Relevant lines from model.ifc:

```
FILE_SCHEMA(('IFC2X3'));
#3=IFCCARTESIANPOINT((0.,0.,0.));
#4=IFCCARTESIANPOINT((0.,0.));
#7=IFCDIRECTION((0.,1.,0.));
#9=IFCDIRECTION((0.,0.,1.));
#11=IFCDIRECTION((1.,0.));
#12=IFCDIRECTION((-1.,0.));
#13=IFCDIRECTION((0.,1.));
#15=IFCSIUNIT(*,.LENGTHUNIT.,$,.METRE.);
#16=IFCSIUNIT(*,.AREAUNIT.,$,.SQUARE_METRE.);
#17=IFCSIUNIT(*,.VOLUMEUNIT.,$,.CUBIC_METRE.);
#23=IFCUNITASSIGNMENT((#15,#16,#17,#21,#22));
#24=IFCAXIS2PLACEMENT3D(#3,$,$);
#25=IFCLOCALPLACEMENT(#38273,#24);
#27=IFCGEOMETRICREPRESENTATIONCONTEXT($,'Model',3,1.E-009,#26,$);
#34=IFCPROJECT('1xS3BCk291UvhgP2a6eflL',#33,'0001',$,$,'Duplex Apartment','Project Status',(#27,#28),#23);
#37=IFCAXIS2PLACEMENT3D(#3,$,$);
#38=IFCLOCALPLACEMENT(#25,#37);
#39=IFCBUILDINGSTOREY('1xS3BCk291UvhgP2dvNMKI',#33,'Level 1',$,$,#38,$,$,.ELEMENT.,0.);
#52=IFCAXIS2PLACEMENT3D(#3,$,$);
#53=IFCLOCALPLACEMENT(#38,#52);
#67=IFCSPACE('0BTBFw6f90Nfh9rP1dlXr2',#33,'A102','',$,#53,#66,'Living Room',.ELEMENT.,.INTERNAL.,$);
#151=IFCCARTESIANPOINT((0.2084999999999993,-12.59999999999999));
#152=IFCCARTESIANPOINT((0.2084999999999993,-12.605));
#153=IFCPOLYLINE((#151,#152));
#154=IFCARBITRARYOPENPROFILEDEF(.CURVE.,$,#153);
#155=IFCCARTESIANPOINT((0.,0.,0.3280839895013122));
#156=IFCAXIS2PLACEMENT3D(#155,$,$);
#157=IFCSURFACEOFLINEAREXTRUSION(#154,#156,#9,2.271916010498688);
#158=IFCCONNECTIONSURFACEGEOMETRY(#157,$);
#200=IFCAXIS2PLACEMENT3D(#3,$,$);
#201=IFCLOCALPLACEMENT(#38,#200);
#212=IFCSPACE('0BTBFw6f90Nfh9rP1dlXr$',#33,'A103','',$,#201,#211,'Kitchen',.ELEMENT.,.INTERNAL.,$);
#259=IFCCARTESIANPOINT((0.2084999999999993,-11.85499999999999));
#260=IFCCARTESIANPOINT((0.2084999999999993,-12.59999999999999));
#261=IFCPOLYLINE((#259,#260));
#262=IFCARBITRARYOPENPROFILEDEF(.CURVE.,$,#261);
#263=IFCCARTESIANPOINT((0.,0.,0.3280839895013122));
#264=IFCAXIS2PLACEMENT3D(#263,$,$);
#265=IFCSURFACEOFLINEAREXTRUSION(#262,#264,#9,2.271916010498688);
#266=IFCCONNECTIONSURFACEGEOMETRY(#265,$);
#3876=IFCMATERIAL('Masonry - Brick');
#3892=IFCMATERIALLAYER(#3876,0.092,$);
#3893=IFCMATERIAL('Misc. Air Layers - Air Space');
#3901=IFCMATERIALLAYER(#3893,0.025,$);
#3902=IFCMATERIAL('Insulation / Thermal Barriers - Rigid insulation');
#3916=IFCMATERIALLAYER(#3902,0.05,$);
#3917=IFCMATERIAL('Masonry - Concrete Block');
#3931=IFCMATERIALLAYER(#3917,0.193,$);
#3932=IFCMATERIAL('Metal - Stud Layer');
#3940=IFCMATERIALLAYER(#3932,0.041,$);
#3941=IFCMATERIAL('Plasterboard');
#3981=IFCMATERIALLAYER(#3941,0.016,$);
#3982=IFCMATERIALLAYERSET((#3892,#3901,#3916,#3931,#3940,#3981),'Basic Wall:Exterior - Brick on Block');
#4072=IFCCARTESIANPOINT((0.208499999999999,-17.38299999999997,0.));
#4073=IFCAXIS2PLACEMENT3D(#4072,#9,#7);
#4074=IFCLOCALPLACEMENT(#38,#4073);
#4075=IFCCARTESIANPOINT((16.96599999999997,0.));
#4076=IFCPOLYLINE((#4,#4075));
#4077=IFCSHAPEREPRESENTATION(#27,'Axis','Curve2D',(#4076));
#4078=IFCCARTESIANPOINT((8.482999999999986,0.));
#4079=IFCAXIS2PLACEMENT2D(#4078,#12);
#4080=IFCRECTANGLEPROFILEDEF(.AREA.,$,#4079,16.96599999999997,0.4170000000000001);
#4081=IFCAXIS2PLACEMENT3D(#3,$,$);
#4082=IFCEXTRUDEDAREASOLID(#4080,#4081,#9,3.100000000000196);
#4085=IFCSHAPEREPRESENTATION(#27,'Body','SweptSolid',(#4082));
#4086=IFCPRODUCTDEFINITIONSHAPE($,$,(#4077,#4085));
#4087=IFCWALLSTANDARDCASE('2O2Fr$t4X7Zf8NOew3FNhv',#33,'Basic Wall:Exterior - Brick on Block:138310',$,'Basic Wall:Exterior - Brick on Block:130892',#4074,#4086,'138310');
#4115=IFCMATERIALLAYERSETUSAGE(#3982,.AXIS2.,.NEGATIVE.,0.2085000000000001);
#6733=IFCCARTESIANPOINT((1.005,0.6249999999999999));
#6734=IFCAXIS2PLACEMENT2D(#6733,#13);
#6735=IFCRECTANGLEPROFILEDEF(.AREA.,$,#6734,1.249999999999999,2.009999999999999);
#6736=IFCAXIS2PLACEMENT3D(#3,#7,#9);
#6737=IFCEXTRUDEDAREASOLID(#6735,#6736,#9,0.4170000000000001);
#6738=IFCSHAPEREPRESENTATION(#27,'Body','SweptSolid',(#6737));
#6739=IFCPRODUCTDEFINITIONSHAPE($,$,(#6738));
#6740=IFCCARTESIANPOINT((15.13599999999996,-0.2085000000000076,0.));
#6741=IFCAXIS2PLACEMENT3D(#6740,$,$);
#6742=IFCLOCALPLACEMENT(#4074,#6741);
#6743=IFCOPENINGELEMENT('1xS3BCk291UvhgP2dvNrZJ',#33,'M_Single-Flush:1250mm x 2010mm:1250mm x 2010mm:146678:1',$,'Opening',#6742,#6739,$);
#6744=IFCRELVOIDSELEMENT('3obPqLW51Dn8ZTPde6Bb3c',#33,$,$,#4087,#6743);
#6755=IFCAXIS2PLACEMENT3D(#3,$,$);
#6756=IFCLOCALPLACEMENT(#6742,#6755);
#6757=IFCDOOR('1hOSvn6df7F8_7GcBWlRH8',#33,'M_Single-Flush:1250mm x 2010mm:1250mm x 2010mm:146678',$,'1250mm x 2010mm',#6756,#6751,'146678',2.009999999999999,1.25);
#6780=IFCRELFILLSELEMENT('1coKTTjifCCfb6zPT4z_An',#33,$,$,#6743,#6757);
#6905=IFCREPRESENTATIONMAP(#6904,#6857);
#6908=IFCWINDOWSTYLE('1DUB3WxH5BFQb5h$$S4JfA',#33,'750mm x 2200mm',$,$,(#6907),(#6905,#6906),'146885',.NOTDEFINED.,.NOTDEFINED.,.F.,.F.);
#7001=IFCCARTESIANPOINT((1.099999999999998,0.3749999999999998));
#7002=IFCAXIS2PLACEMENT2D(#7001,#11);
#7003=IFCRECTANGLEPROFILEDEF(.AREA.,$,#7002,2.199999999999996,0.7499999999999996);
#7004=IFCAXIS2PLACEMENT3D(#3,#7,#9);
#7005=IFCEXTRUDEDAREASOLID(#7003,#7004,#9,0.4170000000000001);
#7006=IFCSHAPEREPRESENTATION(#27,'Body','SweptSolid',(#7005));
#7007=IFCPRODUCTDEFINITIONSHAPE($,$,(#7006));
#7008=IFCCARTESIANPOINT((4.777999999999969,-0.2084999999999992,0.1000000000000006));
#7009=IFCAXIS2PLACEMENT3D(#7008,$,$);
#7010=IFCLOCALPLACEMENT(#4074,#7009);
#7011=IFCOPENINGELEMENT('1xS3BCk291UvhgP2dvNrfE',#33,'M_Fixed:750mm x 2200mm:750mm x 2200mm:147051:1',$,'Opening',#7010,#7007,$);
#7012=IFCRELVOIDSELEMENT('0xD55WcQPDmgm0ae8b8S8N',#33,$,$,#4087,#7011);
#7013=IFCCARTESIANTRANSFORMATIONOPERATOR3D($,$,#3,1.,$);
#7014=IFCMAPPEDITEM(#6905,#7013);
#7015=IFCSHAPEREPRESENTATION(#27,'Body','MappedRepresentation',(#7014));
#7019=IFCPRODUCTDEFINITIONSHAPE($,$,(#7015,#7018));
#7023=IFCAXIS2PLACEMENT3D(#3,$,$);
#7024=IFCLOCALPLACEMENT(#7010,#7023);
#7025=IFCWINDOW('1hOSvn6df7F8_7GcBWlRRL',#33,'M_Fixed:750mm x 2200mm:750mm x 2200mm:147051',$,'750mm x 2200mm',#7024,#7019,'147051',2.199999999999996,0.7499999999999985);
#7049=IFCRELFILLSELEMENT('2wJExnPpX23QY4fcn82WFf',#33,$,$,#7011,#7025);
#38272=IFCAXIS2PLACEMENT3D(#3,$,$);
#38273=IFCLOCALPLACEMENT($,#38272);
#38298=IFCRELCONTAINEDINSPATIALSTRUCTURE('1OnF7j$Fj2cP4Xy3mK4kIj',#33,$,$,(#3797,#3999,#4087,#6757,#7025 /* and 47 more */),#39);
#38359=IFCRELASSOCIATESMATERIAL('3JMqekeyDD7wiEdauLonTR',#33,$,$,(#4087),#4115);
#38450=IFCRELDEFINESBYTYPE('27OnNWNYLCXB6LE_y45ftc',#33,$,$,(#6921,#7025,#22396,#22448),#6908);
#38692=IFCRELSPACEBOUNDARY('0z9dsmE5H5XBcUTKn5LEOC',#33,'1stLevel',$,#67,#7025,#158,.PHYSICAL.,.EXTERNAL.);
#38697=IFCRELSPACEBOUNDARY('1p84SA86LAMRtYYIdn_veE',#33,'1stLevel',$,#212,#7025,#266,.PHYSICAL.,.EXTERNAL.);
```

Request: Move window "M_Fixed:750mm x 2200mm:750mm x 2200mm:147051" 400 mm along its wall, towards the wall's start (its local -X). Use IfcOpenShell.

```python
import numpy as np
import ifcopenshell
import ifcopenshell.api.geometry
import ifcopenshell.util.placement
import ifcopenshell.util.unit

model = ifcopenshell.open("model.ifc")
unit_scale = ifcopenshell.util.unit.calculate_unit_scale(model)

window = model.by_id(7025)
opening = window.FillsVoids[0].RelatingOpeningElement
wall = opening.VoidsElements[0].RelatingBuildingElement

wall_matrix = ifcopenshell.util.placement.get_local_placement(wall.ObjectPlacement)
shift = wall_matrix[:3, 0] * -0.4 / unit_scale
before = ifcopenshell.util.placement.get_local_placement(window.ObjectPlacement)[:3, 3].copy()

# The window is placed relative to its opening, so it follows when the opening moves.
matrix = ifcopenshell.util.placement.get_local_placement(opening.ObjectPlacement)
matrix[:3, 3] += shift
ifcopenshell.api.geometry.edit_object_placement(
    model, product=opening, matrix=matrix, is_si=False, should_transform_children=True
)

# Space boundary surfaces are stored in each space's coordinates; move them too.
for rel in window.ProvidesBoundaries:
    if not rel.ConnectionGeometry:
        continue
    surface = rel.ConnectionGeometry.SurfaceOnRelatingElement
    space_matrix = ifcopenshell.util.placement.get_local_placement(rel.RelatingSpace.ObjectPlacement)
    point = np.array(surface.Position.Location.Coordinates) + space_matrix[:3, :3].T @ shift
    surface.Position = model.createIfcAxis2Placement3D(
        model.createIfcCartesianPoint(point.tolist()), surface.Position.Axis, surface.Position.RefDirection
    )

after = ifcopenshell.util.placement.get_local_placement(window.ObjectPlacement)[:3, 3]
print("window moved by", (after - before).round(3) + 0.0)

model.write("model_updated.ifc")
```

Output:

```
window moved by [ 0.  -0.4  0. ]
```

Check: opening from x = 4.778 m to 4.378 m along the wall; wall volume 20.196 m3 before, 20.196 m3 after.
